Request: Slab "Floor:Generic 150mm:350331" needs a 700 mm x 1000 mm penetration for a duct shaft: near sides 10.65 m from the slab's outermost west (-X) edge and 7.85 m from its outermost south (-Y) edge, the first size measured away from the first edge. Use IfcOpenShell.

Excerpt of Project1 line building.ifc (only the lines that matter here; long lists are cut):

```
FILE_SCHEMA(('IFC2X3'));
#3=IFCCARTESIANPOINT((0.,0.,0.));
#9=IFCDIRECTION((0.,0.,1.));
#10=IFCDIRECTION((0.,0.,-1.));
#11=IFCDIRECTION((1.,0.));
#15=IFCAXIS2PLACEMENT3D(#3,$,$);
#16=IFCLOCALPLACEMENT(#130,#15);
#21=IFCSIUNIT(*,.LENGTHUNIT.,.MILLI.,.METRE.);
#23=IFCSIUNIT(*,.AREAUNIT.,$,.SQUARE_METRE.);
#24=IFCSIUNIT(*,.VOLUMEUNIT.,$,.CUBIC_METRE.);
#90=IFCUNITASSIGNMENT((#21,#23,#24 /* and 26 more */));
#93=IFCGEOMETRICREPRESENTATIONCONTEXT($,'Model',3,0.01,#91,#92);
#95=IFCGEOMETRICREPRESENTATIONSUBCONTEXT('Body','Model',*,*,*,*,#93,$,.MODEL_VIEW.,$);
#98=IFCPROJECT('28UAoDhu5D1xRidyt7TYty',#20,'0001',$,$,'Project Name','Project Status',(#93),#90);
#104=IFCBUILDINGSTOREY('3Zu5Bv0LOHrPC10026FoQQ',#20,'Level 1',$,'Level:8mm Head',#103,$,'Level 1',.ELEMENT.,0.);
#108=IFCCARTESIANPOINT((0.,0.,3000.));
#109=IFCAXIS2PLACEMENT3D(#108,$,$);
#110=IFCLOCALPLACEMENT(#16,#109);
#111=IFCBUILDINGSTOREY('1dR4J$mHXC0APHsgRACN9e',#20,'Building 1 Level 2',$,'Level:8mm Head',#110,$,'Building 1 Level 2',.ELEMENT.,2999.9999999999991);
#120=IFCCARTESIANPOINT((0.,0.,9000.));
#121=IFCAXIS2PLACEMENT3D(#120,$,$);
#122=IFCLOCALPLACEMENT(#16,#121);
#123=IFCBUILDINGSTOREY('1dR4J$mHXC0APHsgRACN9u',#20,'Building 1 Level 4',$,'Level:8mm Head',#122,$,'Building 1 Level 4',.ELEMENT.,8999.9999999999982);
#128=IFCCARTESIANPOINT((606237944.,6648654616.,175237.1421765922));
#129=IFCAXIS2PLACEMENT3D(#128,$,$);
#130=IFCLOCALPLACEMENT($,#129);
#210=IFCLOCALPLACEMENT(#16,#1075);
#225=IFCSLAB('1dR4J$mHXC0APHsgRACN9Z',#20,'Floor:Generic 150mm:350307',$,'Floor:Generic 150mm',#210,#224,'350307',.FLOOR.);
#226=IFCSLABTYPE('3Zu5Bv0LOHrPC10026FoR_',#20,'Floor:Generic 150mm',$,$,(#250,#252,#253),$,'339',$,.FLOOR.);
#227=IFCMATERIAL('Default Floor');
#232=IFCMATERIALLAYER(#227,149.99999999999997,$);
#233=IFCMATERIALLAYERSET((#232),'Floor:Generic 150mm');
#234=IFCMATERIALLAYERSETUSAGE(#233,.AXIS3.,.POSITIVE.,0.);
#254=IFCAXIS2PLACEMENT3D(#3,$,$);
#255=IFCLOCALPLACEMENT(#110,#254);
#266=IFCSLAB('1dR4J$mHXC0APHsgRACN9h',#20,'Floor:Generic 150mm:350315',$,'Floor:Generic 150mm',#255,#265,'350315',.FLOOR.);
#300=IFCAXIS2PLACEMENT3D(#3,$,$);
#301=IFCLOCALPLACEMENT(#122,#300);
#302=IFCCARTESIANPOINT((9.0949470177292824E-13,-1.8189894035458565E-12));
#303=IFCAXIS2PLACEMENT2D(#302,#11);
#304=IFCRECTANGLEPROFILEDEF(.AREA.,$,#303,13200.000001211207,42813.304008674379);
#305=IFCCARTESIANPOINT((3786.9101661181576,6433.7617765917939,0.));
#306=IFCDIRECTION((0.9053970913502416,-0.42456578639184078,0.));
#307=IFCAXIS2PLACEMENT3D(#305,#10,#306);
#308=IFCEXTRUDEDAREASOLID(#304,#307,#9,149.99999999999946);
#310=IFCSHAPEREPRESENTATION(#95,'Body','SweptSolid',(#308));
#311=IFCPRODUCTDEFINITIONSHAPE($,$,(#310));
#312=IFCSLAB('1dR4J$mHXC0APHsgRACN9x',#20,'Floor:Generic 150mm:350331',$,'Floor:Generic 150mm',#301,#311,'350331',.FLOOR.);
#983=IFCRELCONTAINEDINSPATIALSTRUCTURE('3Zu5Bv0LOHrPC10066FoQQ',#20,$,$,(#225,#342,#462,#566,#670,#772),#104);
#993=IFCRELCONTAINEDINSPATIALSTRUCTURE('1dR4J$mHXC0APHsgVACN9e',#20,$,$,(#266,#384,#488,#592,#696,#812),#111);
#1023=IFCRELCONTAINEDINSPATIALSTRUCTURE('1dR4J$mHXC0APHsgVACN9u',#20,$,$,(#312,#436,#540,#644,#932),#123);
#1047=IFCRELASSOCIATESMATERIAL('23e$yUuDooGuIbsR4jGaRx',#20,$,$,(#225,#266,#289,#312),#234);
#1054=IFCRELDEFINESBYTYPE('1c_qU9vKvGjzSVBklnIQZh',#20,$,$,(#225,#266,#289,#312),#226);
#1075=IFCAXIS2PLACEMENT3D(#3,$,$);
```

```python
import numpy as np
import ifcopenshell
import ifcopenshell.api.feature
import ifcopenshell.api.geometry
import ifcopenshell.api.root
import ifcopenshell.geom
import ifcopenshell.util.placement
import ifcopenshell.util.representation
import ifcopenshell.util.shape
import ifcopenshell.util.unit

model = ifcopenshell.open("Project1 line building.ifc")
unit_scale = ifcopenshell.util.unit.calculate_unit_scale(model)
settings = ifcopenshell.geom.settings()


def volume(element):
    """Net volume in cubic metres, openings subtracted."""
    shape = ifcopenshell.geom.create_shape(settings, element)
    return ifcopenshell.util.shape.get_volume(shape.geometry)


slab = model.by_guid("1dR4J$mHXC0APHsgRACN9x")
before = volume(slab)

# Extent in the slab's own axes, in metres. The edges named are its -X and -Y sides.
slab_shape = ifcopenshell.geom.create_shape(settings, slab)
vertices = ifcopenshell.util.shape.get_vertices(slab_shape.geometry)
x_min, y_min, bottom = vertices.min(axis=0)
top = vertices[:, 2].max()

opening = ifcopenshell.api.root.create_entity(model, ifc_class="IfcOpeningElement", name="Duct shaft opening")
context = ifcopenshell.util.representation.get_context(model, "Model", "Body", "MODEL_VIEW")
width, depth = 0.7, 1
outline = [(0.0, 0.0), (width, 0.0), (width, depth), (0.0, depth), (0.0, 0.0)]
# Overshoot both faces by 50 mm so the cut is clean.
shape = ifcopenshell.api.geometry.add_slab_representation(
    model, context=context, depth=top - bottom + 0.1, polyline=outline
)
ifcopenshell.api.geometry.assign_representation(model, product=opening, representation=shape)

matrix = ifcopenshell.util.placement.get_local_placement(slab.ObjectPlacement)
matrix[:, 3] = matrix @ np.append(np.array([x_min + 10.65, y_min + 7.85, bottom - 0.05]) / unit_scale, 1.0)
ifcopenshell.api.geometry.edit_object_placement(model, product=opening, matrix=matrix, is_si=False)
ifcopenshell.api.feature.add_feature(model, feature=opening, element=slab)

after = volume(slab)

print(f"slab volume {before:.3f} -> {after:.3f} m3")

model.write("Project1 line building_rev.ifc")
```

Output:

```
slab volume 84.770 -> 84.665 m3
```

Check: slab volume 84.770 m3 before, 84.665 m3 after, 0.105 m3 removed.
